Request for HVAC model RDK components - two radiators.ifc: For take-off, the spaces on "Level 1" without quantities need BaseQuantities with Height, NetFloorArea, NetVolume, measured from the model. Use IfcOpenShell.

First a look at what the model holds.

```python
import ifcopenshell
import ifcopenshell.util.element
import ifcopenshell.util.unit

model = ifcopenshell.open("HVAC model RDK components - two radiators.ifc")
print(model.schema)
for unit_type in ("LENGTHUNIT", "AREAUNIT", "VOLUMEUNIT"):
    print(unit_type, ifcopenshell.util.unit.calculate_unit_scale(model, unit_type))
storey = next(s for s in model.by_type("IfcBuildingStorey") if s.Name == "Level 1")
spaces = [e for e in ifcopenshell.util.element.get_decomposition(storey) if e.is_a("IfcSpace")]
for e in sorted(spaces, key=lambda e: e.id()):
    print(e.id(), e.is_a(), e.Name, list(ifcopenshell.util.element.get_psets(e, qtos_only=True)), sep=" | ")
```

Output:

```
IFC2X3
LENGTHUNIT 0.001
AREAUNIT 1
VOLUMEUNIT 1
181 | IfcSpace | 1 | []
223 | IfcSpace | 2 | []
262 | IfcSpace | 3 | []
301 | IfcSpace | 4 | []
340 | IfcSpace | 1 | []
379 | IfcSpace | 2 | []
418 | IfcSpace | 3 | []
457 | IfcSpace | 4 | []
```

```python
import ifcopenshell
import ifcopenshell.api.pset
import ifcopenshell.geom
import ifcopenshell.util.element
import ifcopenshell.util.shape
import ifcopenshell.util.unit

model = ifcopenshell.open("HVAC model RDK components - two radiators.ifc")
unit_scale = ifcopenshell.util.unit.calculate_unit_scale(model)
area_scale = ifcopenshell.util.unit.calculate_unit_scale(model, "AREAUNIT")
volume_scale = ifcopenshell.util.unit.calculate_unit_scale(model, "VOLUMEUNIT")
settings = ifcopenshell.geom.settings()

storey = next(s for s in model.by_type("IfcBuildingStorey") if s.Name == "Level 1")
spaces = [e for e in ifcopenshell.util.element.get_decomposition(storey) if e.is_a("IfcSpace")]

for e in sorted(spaces, key=lambda e: e.id()):
    if ifcopenshell.util.element.get_psets(e, qtos_only=True, should_inherit=False):
        continue
    # Geometry comes back in metres, in the element's own axes.
    shape = ifcopenshell.geom.create_shape(settings, e)
    values = {
        "Height": ifcopenshell.util.shape.get_z(shape.geometry) / unit_scale,
        "NetFloorArea": ifcopenshell.util.shape.get_footprint_area(shape.geometry) / area_scale,
        "NetVolume": ifcopenshell.util.shape.get_volume(shape.geometry) / volume_scale,
    }
    qto = ifcopenshell.api.pset.add_qto(model, product=e, name="BaseQuantities")
    ifcopenshell.api.pset.edit_qto(model, qto=qto, properties=values)
    print(e.id(), {k: round(v, 3) for k, v in values.items()})

model.write("HVAC model RDK components - two radiators_updated.ifc")
```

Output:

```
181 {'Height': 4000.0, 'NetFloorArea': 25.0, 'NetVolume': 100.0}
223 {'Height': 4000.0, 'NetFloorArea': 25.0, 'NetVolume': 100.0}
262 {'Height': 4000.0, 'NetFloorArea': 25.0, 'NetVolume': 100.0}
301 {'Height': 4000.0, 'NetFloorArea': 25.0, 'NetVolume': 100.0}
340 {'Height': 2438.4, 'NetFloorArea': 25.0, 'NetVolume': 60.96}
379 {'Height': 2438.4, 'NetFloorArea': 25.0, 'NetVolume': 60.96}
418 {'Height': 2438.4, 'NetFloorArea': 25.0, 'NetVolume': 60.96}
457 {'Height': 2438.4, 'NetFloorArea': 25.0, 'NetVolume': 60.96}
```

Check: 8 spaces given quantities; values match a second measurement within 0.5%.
